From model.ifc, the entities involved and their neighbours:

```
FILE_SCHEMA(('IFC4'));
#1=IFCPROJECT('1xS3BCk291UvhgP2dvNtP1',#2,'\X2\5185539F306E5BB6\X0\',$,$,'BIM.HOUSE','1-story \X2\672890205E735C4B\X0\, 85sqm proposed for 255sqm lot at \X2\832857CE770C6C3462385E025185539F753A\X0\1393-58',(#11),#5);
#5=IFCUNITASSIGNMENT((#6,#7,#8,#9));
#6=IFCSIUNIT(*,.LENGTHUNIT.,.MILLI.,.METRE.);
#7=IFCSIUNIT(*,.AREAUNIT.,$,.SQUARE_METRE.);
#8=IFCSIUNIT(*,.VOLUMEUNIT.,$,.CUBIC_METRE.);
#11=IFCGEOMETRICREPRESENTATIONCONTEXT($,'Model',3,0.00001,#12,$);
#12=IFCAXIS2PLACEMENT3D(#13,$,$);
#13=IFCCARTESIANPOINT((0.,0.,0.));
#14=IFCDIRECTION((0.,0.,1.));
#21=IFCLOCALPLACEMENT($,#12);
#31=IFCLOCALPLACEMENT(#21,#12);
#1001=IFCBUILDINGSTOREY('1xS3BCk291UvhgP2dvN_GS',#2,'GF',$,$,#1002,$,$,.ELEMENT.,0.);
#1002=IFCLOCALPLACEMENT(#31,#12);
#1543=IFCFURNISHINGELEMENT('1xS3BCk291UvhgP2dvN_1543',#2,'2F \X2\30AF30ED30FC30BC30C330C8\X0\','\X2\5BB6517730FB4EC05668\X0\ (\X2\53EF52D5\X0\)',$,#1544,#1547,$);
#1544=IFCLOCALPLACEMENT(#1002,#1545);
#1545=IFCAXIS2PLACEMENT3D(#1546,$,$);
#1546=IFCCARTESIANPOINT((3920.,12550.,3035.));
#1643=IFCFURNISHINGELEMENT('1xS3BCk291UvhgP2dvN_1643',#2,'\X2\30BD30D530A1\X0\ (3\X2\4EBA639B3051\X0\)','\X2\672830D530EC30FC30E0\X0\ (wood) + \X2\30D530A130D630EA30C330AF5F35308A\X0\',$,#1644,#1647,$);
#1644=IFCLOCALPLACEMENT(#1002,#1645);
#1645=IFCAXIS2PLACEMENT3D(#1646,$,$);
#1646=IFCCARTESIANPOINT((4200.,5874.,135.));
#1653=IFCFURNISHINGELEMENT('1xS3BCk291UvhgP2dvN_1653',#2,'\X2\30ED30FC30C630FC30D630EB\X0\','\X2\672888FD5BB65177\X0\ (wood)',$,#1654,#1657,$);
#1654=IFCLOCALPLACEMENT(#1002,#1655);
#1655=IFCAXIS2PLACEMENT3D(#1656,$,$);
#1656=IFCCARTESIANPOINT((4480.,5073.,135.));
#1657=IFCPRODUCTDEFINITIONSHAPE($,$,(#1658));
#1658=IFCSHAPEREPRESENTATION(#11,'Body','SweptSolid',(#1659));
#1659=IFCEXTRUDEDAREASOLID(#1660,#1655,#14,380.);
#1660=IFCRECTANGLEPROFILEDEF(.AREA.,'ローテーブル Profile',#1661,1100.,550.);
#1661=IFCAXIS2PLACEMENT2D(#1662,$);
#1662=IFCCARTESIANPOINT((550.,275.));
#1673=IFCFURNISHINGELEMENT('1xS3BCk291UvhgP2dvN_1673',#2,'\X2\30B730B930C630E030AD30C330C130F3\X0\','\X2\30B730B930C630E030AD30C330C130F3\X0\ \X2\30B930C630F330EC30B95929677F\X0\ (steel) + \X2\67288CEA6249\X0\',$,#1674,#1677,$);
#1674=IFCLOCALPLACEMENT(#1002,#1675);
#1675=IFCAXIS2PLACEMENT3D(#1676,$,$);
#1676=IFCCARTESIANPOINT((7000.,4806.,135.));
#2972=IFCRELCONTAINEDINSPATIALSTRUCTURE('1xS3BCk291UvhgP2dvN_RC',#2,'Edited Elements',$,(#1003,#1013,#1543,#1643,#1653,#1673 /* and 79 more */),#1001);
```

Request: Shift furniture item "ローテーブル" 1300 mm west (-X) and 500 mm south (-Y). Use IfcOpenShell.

```python
import ifcopenshell
import ifcopenshell.api.geometry
import ifcopenshell.util.placement
import ifcopenshell.util.unit

model = ifcopenshell.open("model.ifc")
unit_scale = ifcopenshell.util.unit.calculate_unit_scale(model)

item = model.by_id(1653)
matrix = ifcopenshell.util.placement.get_local_placement(item.ObjectPlacement)
matrix[0, 3] -= 1.3 / unit_scale
matrix[1, 3] -= 0.5 / unit_scale
ifcopenshell.api.geometry.edit_object_placement(model, product=item, matrix=matrix, is_si=False)

print(ifcopenshell.util.placement.get_local_placement(item.ObjectPlacement).round(3) + 0.0)

model.write("model_edited.ifc")
```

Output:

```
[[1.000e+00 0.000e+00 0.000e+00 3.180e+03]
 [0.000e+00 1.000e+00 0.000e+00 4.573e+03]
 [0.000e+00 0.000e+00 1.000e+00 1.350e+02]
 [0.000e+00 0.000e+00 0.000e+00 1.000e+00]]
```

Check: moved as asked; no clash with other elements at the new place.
